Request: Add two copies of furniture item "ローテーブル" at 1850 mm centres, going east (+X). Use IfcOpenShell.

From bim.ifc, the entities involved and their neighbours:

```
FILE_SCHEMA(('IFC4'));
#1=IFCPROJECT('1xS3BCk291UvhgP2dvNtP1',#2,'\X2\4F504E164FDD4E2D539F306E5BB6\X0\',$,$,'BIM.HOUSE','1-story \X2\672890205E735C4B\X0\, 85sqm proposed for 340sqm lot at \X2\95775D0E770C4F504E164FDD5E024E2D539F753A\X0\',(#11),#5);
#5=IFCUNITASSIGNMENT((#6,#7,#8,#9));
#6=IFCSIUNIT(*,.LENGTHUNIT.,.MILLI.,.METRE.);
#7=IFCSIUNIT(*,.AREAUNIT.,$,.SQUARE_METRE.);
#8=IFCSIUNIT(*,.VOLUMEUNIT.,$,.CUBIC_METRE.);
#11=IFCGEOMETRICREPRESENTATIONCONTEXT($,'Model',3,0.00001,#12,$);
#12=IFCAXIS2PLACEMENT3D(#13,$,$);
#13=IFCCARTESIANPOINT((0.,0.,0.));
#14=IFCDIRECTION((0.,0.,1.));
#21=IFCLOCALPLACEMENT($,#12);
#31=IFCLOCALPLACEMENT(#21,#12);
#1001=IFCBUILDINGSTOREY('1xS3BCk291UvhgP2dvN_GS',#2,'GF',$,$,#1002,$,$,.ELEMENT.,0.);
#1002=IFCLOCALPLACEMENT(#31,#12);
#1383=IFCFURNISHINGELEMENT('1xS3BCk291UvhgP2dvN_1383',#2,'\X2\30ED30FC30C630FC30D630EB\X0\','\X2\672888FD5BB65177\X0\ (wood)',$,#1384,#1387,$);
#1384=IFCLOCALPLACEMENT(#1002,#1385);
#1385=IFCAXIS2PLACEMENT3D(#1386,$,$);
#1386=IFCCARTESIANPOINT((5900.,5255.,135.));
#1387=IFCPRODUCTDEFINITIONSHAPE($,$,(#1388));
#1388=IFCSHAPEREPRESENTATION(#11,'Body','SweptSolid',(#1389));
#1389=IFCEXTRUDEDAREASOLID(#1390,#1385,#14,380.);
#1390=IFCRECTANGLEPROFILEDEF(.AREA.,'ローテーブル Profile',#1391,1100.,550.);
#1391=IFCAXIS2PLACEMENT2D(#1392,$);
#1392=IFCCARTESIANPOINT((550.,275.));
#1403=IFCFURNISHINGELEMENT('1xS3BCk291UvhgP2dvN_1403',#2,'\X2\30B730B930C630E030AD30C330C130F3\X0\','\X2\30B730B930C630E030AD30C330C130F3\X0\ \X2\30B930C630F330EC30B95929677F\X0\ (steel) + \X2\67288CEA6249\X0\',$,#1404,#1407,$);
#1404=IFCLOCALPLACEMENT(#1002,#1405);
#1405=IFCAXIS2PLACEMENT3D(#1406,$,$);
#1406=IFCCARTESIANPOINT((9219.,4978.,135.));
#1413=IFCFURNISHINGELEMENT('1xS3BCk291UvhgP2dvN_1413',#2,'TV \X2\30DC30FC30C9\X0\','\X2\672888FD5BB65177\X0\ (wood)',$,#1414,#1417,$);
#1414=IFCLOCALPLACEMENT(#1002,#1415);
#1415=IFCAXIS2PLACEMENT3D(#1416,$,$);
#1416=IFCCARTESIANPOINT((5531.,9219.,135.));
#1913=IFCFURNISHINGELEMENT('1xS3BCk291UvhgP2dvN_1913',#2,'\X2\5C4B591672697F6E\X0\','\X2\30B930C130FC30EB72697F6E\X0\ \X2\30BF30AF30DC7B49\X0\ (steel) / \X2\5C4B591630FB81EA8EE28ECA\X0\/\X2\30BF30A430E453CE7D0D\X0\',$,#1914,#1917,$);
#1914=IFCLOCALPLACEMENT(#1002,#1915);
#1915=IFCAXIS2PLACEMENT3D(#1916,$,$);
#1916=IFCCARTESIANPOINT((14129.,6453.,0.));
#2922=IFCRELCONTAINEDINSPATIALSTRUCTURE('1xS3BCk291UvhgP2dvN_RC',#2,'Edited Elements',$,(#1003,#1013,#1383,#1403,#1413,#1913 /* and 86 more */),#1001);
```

```python
import numpy as np
import ifcopenshell
import ifcopenshell.api.geometry
import ifcopenshell.api.root
import ifcopenshell.util.element
import ifcopenshell.util.placement
import ifcopenshell.util.unit

model = ifcopenshell.open("bim.ifc")
unit_scale = ifcopenshell.util.unit.calculate_unit_scale(model)


def reuse_history(source, copy):
    """copy_class also copies each property set's owner history, people and application; keep the originals."""
    for rel in copy.IsDefinedBy:
        if rel.is_a("IfcRelDefinesByProperties") and (history := rel.RelatingPropertyDefinition.OwnerHistory):
            rel.RelatingPropertyDefinition.OwnerHistory = source.OwnerHistory
            ifcopenshell.util.element.remove_deep2(model, history)


source = model.by_guid("1xS3BCk291UvhgP2dvN_1383")
base = ifcopenshell.util.placement.get_local_placement(source.ObjectPlacement)
step = np.array([1.0, 0.0, 0.0]) * 1.85 / unit_scale

for i in range(1, 3):
    copy = ifcopenshell.api.root.copy_class(model, product=source)
    copy.Representation = ifcopenshell.util.element.copy_deep(
        model, source.Representation, exclude=["IfcGeometricRepresentationContext", "IfcRepresentationMap"]
    )
    reuse_history(source, copy)
    matrix = base.copy()
    matrix[:3, 3] += i * step
    print("added at", matrix[:3, 3].round(3) + 0.0)
    ifcopenshell.api.geometry.edit_object_placement(model, product=copy, matrix=matrix, is_si=False)

model.write("bim_v2.ifc")
```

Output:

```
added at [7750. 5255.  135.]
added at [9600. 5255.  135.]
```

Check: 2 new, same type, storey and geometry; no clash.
